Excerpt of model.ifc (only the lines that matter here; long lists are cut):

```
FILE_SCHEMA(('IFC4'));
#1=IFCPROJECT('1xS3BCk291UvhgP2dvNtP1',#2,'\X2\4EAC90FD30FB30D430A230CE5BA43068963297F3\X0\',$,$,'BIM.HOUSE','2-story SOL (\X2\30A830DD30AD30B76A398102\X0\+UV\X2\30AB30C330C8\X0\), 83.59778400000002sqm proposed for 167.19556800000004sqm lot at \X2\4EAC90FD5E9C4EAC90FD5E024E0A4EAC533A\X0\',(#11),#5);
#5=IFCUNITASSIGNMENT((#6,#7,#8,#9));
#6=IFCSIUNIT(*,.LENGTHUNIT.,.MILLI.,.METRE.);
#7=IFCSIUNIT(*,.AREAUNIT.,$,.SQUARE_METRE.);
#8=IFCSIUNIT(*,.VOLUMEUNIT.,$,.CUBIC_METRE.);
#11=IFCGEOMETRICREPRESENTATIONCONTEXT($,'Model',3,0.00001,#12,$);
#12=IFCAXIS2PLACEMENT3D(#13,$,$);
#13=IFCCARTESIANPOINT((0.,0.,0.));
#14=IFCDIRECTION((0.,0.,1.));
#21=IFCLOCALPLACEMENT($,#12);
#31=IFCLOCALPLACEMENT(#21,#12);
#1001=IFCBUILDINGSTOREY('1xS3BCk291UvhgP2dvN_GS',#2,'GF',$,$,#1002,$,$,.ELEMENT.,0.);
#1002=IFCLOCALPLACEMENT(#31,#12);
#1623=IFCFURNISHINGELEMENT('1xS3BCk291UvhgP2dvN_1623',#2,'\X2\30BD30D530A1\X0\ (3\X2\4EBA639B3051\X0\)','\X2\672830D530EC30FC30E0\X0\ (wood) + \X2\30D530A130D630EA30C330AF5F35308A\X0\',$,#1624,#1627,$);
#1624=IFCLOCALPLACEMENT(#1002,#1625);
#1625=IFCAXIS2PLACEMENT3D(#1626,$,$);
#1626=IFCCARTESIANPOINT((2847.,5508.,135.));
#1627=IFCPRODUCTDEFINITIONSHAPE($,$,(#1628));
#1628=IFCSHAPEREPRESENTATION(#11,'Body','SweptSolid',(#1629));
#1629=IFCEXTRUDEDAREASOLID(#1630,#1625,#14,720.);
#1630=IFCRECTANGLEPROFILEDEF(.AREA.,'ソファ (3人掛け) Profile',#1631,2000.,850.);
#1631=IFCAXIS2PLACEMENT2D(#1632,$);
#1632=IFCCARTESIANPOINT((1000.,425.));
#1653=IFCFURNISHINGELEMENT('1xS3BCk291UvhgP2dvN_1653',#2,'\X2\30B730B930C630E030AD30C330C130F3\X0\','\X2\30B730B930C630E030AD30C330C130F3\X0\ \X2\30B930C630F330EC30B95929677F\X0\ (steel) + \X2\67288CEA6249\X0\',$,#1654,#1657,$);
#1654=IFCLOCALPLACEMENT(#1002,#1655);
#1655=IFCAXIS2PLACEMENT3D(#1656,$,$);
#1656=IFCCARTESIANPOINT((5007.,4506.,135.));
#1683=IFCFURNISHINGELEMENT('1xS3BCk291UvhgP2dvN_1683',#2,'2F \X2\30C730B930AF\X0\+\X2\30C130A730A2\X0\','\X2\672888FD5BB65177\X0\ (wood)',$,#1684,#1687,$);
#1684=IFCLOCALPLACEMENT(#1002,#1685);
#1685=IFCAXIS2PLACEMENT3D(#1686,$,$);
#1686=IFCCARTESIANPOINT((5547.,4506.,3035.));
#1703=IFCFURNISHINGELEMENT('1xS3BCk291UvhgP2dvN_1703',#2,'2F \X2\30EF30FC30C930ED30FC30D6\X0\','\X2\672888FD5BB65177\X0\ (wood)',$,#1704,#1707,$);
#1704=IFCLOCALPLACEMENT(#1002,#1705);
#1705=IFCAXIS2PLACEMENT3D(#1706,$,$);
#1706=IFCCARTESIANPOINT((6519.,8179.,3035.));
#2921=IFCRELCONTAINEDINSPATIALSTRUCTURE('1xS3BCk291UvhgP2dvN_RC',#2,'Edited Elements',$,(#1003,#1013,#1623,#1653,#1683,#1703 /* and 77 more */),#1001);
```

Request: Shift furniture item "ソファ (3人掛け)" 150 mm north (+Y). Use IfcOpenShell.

```python
import ifcopenshell
import ifcopenshell.api.geometry
import ifcopenshell.util.placement
import ifcopenshell.util.unit

model = ifcopenshell.open("model.ifc")
unit_scale = ifcopenshell.util.unit.calculate_unit_scale(model)

item = model.by_guid("1xS3BCk291UvhgP2dvN_1623")
matrix = ifcopenshell.util.placement.get_local_placement(item.ObjectPlacement)
matrix[1, 3] += 0.15 / unit_scale
ifcopenshell.api.geometry.edit_object_placement(model, product=item, matrix=matrix, is_si=False)

print(ifcopenshell.util.placement.get_local_placement(item.ObjectPlacement).round(3) + 0.0)

model.write("model_edited.ifc")
```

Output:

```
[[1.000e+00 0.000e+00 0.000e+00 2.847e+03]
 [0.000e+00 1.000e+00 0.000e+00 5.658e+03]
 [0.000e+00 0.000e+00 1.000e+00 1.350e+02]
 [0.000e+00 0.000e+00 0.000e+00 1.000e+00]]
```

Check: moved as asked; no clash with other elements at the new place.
